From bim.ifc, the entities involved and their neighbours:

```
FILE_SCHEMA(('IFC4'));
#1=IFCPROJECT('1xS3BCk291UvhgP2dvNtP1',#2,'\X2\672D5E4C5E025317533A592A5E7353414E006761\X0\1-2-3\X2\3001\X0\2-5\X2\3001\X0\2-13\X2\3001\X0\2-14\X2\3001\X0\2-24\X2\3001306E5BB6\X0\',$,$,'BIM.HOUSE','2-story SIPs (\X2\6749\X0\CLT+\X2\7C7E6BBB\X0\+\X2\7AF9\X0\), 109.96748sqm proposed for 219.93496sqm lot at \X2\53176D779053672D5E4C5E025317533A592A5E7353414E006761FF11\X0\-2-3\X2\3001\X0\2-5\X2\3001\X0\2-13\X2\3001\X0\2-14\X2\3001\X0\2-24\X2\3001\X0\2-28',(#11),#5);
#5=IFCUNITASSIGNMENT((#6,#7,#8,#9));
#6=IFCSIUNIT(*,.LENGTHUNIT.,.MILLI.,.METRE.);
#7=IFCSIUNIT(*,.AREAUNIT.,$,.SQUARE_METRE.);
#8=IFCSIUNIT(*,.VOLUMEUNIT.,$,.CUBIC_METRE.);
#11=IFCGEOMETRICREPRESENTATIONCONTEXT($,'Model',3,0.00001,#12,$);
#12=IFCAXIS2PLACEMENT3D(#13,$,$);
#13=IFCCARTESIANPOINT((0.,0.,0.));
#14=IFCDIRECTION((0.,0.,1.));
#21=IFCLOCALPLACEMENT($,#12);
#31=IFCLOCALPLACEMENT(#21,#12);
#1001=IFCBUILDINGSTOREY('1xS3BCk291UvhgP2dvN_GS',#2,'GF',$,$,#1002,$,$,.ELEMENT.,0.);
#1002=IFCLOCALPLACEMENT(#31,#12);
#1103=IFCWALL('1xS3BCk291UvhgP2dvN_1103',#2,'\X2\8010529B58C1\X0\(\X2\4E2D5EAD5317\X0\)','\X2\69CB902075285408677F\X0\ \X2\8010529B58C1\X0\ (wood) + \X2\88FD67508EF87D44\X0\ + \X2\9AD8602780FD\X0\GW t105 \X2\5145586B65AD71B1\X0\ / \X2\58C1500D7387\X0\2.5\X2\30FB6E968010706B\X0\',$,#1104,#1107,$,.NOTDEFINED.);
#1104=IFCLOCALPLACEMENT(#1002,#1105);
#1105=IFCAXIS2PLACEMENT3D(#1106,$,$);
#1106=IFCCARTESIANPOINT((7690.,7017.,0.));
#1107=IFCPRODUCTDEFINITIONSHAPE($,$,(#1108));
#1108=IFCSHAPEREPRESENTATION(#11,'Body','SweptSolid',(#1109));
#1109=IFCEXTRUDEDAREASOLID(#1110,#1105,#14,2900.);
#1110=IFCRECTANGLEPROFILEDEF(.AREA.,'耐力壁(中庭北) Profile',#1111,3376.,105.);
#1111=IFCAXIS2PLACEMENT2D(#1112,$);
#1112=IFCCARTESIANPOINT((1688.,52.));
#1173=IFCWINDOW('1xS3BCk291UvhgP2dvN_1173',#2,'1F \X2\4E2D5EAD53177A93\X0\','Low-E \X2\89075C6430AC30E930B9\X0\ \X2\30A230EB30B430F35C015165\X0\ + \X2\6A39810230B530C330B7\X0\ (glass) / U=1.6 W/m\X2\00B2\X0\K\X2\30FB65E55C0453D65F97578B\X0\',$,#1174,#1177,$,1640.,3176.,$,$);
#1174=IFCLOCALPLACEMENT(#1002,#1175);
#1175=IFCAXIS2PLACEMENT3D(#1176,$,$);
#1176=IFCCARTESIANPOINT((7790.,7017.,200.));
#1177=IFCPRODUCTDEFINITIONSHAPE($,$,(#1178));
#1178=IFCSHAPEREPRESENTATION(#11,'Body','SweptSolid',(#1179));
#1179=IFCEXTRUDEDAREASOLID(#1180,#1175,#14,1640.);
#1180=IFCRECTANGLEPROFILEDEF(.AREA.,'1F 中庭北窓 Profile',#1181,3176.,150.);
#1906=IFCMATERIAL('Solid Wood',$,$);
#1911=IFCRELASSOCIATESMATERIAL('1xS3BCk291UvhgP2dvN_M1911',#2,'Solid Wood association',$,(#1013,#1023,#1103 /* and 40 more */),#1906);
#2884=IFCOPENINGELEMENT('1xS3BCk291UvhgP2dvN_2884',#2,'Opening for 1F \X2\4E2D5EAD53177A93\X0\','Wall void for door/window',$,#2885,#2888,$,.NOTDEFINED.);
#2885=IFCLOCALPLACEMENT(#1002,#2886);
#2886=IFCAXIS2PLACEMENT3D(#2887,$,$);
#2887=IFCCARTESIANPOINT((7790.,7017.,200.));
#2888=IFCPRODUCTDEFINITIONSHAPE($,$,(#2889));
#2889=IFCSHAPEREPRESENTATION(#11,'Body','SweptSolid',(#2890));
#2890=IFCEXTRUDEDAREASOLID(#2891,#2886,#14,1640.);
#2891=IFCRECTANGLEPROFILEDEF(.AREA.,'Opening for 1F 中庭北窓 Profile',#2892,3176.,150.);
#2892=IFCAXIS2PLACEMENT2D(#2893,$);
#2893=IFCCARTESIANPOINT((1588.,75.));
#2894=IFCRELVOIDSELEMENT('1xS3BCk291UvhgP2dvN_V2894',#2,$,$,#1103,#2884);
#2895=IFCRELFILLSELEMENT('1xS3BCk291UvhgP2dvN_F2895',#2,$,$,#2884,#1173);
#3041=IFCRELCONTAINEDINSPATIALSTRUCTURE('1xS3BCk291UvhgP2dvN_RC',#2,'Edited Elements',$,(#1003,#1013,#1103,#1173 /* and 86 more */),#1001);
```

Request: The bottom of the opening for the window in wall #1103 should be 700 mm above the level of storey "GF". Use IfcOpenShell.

```python
import numpy as np
import ifcopenshell
import ifcopenshell.api.geometry
import ifcopenshell.geom
import ifcopenshell.util.element
import ifcopenshell.util.placement
import ifcopenshell.util.shape
import ifcopenshell.util.unit

model = ifcopenshell.open("bim.ifc")
unit_scale = ifcopenshell.util.unit.calculate_unit_scale(model)

window = model.by_guid("1xS3BCk291UvhgP2dvN_1173")
opening = window.FillsVoids[0].RelatingOpeningElement
storey = ifcopenshell.util.element.get_container(window, ifc_class="IfcBuildingStorey")
level = ifcopenshell.util.placement.get_local_placement(storey.ObjectPlacement)[2, 3]

# The opening's origin need not be at the sill, so measure its lowest point.
shape = ifcopenshell.geom.create_shape(ifcopenshell.geom.settings(), opening)
bottom = ifcopenshell.util.shape.get_shape_bottom_elevation(shape, shape.geometry) / unit_scale
dz = level + 0.7 / unit_scale - bottom

shift = np.array([0.0, 0.0, dz])
# The window is not placed relative to its opening, so move both.
for product in (opening, window):
    matrix = ifcopenshell.util.placement.get_local_placement(product.ObjectPlacement)
    matrix[:3, 3] += shift
    ifcopenshell.api.geometry.edit_object_placement(model, product=product, matrix=matrix, is_si=False)

print(f"moved by {dz * unit_scale:+.3f} m")

model.write("bim_v2.ifc")
```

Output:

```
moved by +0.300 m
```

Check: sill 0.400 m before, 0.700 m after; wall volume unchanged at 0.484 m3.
